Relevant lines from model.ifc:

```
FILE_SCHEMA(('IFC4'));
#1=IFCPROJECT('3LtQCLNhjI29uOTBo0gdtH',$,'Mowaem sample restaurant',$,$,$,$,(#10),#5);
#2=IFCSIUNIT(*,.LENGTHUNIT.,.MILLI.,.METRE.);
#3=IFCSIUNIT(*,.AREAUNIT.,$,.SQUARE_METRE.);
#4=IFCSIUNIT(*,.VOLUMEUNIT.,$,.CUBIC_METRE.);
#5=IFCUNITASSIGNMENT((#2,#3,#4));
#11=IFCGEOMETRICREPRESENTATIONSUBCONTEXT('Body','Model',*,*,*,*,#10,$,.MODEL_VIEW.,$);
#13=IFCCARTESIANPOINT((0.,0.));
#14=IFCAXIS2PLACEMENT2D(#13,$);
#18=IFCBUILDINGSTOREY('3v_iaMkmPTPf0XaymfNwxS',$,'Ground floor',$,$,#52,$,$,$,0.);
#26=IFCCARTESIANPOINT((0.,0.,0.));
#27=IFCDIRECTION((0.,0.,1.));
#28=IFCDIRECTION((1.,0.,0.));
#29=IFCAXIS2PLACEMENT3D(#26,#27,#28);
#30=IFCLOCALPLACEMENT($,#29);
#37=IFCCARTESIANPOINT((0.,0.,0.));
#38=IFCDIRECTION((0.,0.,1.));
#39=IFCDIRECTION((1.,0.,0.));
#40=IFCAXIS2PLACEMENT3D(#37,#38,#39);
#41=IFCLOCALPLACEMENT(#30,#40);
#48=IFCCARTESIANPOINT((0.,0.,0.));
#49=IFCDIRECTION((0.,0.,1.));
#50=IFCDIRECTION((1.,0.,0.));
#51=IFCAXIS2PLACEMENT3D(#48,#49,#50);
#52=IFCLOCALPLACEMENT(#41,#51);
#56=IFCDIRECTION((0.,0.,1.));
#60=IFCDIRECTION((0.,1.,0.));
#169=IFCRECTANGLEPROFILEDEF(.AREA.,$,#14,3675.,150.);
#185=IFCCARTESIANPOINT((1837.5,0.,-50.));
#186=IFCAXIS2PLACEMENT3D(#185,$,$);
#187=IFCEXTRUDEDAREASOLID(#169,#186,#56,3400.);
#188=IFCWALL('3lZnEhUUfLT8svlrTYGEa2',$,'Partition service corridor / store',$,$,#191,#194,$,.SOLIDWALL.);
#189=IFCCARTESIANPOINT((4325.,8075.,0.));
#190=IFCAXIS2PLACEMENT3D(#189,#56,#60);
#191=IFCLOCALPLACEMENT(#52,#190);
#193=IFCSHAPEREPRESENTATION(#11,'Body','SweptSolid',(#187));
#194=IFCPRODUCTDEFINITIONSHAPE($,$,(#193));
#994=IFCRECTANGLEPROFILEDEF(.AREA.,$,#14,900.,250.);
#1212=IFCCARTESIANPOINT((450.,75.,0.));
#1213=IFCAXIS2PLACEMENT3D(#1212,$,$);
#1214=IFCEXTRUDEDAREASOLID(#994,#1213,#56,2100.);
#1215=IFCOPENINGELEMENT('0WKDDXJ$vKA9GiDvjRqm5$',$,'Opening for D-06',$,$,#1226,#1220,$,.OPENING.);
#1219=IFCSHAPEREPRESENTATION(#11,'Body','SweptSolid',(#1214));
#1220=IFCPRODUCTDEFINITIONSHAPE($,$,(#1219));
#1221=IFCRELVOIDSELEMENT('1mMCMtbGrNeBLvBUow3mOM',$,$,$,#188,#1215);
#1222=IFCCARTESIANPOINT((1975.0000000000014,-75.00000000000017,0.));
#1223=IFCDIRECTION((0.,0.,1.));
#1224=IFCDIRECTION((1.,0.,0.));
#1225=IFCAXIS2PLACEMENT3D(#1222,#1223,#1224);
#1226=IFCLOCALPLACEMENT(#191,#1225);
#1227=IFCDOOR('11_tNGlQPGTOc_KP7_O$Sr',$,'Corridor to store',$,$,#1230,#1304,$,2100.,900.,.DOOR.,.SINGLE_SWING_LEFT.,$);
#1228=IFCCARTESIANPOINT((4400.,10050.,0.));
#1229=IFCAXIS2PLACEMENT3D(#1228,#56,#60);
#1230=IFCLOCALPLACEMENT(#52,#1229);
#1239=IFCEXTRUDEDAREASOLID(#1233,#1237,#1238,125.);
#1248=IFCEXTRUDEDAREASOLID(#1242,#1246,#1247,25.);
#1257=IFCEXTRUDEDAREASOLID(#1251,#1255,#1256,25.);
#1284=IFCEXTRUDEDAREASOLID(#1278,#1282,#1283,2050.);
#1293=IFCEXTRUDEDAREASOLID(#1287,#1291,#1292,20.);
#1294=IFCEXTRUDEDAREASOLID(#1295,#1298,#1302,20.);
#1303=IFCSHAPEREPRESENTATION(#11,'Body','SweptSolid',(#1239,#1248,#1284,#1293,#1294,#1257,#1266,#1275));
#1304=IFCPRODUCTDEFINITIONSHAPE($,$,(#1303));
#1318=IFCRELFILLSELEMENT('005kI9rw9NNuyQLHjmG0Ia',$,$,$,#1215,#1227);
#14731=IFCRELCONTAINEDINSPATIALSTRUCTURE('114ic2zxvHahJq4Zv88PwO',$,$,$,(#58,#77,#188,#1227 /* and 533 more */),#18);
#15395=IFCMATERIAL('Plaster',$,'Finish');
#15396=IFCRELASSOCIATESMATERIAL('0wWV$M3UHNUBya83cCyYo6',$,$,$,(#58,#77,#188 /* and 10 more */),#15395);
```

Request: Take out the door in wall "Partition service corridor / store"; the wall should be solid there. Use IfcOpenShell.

```python
import ifcopenshell
import ifcopenshell.api.feature
import ifcopenshell.api.root
import ifcopenshell.geom
import ifcopenshell.util.shape

model = ifcopenshell.open("model.ifc")
settings = ifcopenshell.geom.settings()


def volume(element):
    """Net volume in cubic metres, openings subtracted."""
    shape = ifcopenshell.geom.create_shape(settings, element)
    return ifcopenshell.util.shape.get_volume(shape.geometry)


door = model.by_guid("11_tNGlQPGTOc_KP7_O$Sr")
opening = door.FillsVoids[0].RelatingOpeningElement
wall = opening.VoidsElements[0].RelatingBuildingElement
before = volume(wall)

ifcopenshell.api.root.remove_product(model, product=door)
ifcopenshell.api.feature.remove_feature(model, feature=opening)

after = volume(wall)

print(f"wall volume {before:.3f} -> {after:.3f} m3")

model.write("model-out.ifc")
```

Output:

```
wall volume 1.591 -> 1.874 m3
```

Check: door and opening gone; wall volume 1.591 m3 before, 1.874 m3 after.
